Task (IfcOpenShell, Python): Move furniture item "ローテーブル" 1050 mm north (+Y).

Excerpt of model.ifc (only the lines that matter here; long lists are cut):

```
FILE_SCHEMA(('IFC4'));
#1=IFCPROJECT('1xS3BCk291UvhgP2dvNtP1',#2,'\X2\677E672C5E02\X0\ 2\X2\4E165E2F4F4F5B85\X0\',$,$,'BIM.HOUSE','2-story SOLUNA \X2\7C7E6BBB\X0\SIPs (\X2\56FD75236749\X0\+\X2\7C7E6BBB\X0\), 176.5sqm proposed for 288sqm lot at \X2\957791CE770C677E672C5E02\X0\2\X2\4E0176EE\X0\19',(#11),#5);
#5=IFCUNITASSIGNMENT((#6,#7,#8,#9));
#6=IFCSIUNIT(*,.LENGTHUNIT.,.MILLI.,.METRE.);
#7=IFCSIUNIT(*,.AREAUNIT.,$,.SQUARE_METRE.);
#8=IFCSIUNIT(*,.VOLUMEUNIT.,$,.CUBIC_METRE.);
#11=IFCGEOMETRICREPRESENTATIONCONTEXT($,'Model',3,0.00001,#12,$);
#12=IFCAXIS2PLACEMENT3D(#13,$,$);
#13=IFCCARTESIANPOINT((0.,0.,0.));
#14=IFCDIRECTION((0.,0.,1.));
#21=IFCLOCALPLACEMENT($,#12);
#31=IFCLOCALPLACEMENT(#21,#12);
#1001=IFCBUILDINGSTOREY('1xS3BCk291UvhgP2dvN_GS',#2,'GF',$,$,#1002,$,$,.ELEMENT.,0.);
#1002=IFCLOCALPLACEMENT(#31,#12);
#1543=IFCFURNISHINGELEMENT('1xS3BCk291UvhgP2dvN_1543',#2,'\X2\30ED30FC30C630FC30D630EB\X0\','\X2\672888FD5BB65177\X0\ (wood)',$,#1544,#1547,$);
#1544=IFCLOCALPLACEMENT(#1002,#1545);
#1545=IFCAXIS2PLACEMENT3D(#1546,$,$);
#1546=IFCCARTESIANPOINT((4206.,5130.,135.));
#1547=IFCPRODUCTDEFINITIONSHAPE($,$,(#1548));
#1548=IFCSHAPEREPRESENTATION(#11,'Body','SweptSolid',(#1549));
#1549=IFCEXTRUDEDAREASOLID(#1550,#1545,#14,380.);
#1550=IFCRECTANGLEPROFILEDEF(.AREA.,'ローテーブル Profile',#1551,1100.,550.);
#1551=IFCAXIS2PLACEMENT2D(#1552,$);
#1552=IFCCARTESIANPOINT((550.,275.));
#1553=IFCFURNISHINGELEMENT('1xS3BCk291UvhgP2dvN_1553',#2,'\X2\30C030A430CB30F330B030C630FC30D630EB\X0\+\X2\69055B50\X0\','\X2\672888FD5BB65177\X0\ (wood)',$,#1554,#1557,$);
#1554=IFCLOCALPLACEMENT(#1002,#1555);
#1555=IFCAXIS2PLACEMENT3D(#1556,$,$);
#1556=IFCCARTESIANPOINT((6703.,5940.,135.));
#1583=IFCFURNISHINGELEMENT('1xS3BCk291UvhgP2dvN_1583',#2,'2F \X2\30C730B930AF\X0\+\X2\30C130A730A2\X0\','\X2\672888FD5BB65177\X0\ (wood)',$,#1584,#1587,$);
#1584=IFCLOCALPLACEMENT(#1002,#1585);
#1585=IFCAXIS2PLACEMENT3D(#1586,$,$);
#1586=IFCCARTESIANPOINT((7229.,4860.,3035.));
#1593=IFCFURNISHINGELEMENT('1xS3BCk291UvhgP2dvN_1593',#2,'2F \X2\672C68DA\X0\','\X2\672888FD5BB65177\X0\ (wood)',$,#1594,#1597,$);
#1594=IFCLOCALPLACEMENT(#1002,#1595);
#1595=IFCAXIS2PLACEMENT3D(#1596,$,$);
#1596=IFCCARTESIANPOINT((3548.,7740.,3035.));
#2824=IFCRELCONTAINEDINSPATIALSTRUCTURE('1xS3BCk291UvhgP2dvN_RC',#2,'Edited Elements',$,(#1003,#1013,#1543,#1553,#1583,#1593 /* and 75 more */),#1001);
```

```python
import ifcopenshell
import ifcopenshell.api.geometry
import ifcopenshell.util.placement
import ifcopenshell.util.unit

model = ifcopenshell.open("model.ifc")
unit_scale = ifcopenshell.util.unit.calculate_unit_scale(model)

item = model.by_guid("1xS3BCk291UvhgP2dvN_1543")
matrix = ifcopenshell.util.placement.get_local_placement(item.ObjectPlacement)
matrix[1, 3] += 1.05 / unit_scale
ifcopenshell.api.geometry.edit_object_placement(model, product=item, matrix=matrix, is_si=False)

print(ifcopenshell.util.placement.get_local_placement(item.ObjectPlacement).round(3) + 0.0)

model.write("model-out.ifc")
```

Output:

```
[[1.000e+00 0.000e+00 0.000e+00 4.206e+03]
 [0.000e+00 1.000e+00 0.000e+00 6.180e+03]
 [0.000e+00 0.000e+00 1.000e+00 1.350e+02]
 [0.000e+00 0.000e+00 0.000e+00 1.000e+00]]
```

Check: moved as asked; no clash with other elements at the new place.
